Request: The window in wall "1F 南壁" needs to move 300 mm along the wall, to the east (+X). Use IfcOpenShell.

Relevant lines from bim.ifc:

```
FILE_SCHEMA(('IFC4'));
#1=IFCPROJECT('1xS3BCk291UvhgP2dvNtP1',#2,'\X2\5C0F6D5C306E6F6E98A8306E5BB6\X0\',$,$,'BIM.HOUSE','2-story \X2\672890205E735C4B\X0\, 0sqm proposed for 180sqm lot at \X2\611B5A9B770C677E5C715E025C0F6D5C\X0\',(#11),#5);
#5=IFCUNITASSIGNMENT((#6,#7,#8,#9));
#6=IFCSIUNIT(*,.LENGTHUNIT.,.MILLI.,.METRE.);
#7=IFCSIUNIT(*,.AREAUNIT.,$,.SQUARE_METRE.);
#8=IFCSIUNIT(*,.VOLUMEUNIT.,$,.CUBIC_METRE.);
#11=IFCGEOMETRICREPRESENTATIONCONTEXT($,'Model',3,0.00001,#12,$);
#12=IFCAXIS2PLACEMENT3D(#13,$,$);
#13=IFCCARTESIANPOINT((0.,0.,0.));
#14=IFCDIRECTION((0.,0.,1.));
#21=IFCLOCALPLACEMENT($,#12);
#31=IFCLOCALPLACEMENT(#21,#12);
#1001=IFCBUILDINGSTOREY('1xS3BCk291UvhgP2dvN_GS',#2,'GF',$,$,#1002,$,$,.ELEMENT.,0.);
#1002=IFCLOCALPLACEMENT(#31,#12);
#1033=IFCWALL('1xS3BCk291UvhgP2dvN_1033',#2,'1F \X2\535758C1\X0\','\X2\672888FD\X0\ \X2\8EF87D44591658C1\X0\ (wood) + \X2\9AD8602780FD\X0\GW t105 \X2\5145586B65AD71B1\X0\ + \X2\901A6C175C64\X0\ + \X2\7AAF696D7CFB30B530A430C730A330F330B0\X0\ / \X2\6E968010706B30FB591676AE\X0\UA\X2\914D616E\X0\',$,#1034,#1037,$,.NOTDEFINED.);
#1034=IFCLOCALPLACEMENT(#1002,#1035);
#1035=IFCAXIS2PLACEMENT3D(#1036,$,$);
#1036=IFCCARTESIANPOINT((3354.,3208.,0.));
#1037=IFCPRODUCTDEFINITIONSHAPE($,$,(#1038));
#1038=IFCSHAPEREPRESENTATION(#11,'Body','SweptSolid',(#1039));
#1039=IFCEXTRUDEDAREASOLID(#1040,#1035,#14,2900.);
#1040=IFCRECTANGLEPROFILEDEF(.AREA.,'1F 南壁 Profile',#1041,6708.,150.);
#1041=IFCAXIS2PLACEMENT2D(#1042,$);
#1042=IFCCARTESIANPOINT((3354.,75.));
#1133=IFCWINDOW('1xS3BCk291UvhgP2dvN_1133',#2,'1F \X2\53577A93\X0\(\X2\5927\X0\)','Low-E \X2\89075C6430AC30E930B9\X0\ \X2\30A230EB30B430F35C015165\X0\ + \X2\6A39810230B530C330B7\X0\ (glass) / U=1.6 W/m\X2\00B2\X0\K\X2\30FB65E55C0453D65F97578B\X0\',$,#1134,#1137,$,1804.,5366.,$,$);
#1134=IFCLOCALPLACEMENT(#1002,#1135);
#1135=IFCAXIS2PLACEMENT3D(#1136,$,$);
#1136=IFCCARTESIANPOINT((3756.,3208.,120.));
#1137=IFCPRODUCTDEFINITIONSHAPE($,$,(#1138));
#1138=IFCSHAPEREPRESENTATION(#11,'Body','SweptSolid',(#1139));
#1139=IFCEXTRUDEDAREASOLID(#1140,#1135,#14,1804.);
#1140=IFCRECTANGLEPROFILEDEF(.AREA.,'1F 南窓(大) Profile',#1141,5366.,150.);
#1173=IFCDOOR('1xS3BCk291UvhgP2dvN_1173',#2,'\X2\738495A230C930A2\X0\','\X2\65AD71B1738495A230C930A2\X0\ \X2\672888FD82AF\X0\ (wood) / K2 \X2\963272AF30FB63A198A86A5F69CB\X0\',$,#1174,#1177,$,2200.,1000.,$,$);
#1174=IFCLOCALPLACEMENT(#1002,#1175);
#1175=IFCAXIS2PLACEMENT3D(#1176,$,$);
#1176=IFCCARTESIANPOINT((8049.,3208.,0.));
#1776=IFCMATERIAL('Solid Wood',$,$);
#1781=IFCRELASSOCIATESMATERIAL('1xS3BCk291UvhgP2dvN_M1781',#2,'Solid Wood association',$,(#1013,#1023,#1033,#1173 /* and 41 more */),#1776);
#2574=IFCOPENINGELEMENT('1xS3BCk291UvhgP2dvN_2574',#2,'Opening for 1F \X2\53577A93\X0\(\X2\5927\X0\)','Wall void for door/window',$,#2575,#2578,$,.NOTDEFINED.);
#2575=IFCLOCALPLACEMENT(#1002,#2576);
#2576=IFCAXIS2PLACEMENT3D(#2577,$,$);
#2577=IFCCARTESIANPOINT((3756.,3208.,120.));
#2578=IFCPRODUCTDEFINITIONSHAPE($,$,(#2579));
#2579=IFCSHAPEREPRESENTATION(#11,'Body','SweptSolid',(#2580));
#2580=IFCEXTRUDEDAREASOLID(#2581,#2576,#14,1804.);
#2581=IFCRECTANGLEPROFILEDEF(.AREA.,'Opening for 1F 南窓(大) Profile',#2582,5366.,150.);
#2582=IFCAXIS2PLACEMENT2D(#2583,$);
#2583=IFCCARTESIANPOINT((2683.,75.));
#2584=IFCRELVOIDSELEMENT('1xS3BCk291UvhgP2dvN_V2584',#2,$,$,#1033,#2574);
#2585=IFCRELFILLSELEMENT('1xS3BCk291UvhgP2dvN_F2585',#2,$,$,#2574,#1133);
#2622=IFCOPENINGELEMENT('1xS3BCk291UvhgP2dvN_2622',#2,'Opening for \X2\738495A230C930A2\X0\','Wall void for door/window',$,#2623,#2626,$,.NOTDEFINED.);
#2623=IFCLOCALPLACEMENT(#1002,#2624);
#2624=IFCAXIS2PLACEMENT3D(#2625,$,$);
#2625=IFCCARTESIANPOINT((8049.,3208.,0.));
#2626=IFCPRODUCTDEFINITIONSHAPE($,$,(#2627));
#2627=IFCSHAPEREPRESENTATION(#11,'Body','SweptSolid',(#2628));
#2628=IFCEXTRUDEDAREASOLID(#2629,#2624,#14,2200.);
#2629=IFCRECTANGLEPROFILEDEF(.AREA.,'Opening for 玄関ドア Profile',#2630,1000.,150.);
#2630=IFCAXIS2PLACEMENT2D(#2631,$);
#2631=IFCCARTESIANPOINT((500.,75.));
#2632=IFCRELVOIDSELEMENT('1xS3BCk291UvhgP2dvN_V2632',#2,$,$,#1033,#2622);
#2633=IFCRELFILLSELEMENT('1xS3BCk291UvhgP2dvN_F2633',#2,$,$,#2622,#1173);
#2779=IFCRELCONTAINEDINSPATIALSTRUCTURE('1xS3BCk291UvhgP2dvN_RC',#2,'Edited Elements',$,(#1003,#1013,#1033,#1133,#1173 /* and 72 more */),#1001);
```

```python
import ifcopenshell
import ifcopenshell.api.geometry
import ifcopenshell.util.placement
import ifcopenshell.util.unit

model = ifcopenshell.open("bim.ifc")
unit_scale = ifcopenshell.util.unit.calculate_unit_scale(model)

window = model.by_guid("1xS3BCk291UvhgP2dvN_1133")
opening = window.FillsVoids[0].RelatingOpeningElement
wall = opening.VoidsElements[0].RelatingBuildingElement

wall_matrix = ifcopenshell.util.placement.get_local_placement(wall.ObjectPlacement)
shift = wall_matrix[:3, 0] * 0.3 / unit_scale
before = ifcopenshell.util.placement.get_local_placement(window.ObjectPlacement)[:3, 3].copy()

# The window is not placed relative to its opening, so move both.
for product in (opening, window):
    matrix = ifcopenshell.util.placement.get_local_placement(product.ObjectPlacement)
    matrix[:3, 3] += shift
    ifcopenshell.api.geometry.edit_object_placement(model, product=product, matrix=matrix, is_si=False)

after = ifcopenshell.util.placement.get_local_placement(window.ObjectPlacement)[:3, 3]
print("window moved by", (after - before).round(3) + 0.0)

model.write("bim_edited.ifc")
```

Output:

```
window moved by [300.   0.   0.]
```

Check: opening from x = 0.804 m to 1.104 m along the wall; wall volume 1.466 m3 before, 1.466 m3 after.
